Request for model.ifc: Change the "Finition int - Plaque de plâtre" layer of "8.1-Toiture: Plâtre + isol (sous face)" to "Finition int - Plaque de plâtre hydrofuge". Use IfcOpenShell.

First a look at what the model holds.

```python
import ifcopenshell
import ifcopenshell.util.element

model = ifcopenshell.open("model.ifc")
print(model.schema)
for layer_set in model.by_type("IfcMaterialLayerSet"):
    if layer_set.LayerSetName == "8.1-Toiture: Plâtre + isol (sous face)":
        for layer in layer_set.MaterialLayers:
            print(layer.id(), layer.Material and layer.Material.Name, layer.LayerThickness, sep=" | ")
        print(len(ifcopenshell.util.element.get_elements_by_material(model, layer_set)), "elements and types use it")
print(sorted(m.Name for m in model.by_type("IfcMaterial") if m.Name)[:60])
```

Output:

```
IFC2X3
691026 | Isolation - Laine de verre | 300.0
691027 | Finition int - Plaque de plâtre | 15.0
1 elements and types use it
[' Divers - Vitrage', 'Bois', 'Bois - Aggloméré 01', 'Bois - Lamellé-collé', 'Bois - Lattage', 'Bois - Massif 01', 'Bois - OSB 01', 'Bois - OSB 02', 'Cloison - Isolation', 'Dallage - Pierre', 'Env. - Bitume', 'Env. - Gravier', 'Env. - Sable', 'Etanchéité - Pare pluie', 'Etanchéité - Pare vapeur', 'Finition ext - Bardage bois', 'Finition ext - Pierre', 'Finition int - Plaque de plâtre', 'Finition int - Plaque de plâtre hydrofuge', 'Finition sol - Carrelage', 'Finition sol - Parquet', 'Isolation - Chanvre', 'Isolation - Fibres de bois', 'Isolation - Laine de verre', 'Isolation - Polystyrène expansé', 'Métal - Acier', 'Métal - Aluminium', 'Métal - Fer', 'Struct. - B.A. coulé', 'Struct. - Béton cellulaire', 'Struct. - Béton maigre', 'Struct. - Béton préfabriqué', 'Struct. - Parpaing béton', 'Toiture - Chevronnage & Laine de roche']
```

```python
import ifcopenshell
import ifcopenshell.api.material

model = ifcopenshell.open("model.ifc")

layer_set = next(s for s in model.by_type("IfcMaterialLayerSet") if s.LayerSetName == "8.1-Toiture: Plâtre + isol (sous face)")
layer = next(l for l in layer_set.MaterialLayers if l.Material and l.Material.Name == "Finition int - Plaque de plâtre")
material = next(m for m in model.by_type("IfcMaterial") if m.Name == "Finition int - Plaque de plâtre hydrofuge")

# Point this one layer at the other material; renaming the old one would change it everywhere.
ifcopenshell.api.material.edit_layer(model, layer=layer, attributes={}, material=material)

print([l.Material.Name if l.Material else None for l in layer_set.MaterialLayers])

model.write("model-out.ifc")
```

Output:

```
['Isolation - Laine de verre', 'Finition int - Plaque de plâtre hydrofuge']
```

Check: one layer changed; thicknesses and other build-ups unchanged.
